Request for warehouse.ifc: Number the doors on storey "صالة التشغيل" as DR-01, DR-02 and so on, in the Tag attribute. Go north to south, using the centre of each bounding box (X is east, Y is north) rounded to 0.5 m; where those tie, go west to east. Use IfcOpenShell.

First a look at what the model holds.

```python
import ifcopenshell
import ifcopenshell.util.element
import ifcopenshell.util.placement

model = ifcopenshell.open("warehouse.ifc")
print(model.schema)
storey = next(s for s in model.by_type("IfcBuildingStorey") if s.Name == "صالة التشغيل")
doors = [e for e in ifcopenshell.util.element.get_decomposition(storey) if e.is_a("IfcDoor")]
for e in sorted(doors, key=lambda e: e.id()):
    origin = ifcopenshell.util.placement.get_local_placement(e.ObjectPlacement)[:3, 3]
    print(e.id(), e.Tag, e.Name, origin.round(2) + 0.0, sep=" | ")
```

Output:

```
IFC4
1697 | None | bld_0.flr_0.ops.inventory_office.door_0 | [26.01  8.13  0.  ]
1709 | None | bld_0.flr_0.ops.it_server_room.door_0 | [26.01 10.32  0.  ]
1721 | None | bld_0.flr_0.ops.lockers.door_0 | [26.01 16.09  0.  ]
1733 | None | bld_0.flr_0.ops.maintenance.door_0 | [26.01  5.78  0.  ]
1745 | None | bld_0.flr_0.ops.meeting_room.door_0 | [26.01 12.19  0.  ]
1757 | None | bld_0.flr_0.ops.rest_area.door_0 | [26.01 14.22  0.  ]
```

```python
import ifcopenshell
import ifcopenshell.geom
import ifcopenshell.util.element
import ifcopenshell.util.shape

model = ifcopenshell.open("warehouse.ifc")
settings = ifcopenshell.geom.settings()
settings.set("use-world-coords", True)


def centre(element):
    shape = ifcopenshell.geom.create_shape(settings, element)
    return ifcopenshell.util.shape.get_bbox_centroid(shape.geometry)


storey = next(s for s in model.by_type("IfcBuildingStorey") if s.Name == "صالة التشغيل")
doors = [e for e in ifcopenshell.util.element.get_decomposition(storey) if e.is_a("IfcDoor")]

# Insertion points can sit at a corner or the storey origin, so sort by the geometry (in metres).
centres = {e: centre(e) for e in doors}
doors.sort(key=lambda e: (-round(centres[e][1] / 0.5), centres[e][0]))

for i, e in enumerate(doors, start=1):
    number = f"DR-{i:02d}"
    e.Tag = number
    print(e.id(), number)

model.write("warehouse_updated.ifc")
```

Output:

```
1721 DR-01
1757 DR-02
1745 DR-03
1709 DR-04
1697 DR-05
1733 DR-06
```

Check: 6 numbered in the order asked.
